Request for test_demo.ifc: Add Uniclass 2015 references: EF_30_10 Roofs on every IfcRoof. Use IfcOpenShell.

First a look at what the model holds.

```python
import ifcopenshell

model = ifcopenshell.open("test_demo.ifc")
print(model.schema)
print("classifications:", [c.Name for c in model.by_type("IfcClassification")])
for ifc_class in ("IfcDoor", "IfcRoof", "IfcStair", "IfcWall", "IfcWindow"):
    print(ifc_class, len(model.by_type(ifc_class)))
```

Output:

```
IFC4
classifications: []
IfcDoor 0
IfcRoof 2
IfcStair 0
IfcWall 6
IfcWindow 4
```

```python
import ifcopenshell
import ifcopenshell.api.classification

model = ifcopenshell.open("test_demo.ifc")

system = ifcopenshell.api.classification.add_classification(model, classification="Uniclass 2015")

codes = {
    "IfcRoof": ("EF_30_10", "Roofs"),
}
for ifc_class, (code, name) in codes.items():
    products = model.by_type(ifc_class)
    ifcopenshell.api.classification.add_reference(
        model, products=products, classification=system, identification=code, name=name
    )
    print(code, len(products))

model.write("test_demo_updated.ifc")
```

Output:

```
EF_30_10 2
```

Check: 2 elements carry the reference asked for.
